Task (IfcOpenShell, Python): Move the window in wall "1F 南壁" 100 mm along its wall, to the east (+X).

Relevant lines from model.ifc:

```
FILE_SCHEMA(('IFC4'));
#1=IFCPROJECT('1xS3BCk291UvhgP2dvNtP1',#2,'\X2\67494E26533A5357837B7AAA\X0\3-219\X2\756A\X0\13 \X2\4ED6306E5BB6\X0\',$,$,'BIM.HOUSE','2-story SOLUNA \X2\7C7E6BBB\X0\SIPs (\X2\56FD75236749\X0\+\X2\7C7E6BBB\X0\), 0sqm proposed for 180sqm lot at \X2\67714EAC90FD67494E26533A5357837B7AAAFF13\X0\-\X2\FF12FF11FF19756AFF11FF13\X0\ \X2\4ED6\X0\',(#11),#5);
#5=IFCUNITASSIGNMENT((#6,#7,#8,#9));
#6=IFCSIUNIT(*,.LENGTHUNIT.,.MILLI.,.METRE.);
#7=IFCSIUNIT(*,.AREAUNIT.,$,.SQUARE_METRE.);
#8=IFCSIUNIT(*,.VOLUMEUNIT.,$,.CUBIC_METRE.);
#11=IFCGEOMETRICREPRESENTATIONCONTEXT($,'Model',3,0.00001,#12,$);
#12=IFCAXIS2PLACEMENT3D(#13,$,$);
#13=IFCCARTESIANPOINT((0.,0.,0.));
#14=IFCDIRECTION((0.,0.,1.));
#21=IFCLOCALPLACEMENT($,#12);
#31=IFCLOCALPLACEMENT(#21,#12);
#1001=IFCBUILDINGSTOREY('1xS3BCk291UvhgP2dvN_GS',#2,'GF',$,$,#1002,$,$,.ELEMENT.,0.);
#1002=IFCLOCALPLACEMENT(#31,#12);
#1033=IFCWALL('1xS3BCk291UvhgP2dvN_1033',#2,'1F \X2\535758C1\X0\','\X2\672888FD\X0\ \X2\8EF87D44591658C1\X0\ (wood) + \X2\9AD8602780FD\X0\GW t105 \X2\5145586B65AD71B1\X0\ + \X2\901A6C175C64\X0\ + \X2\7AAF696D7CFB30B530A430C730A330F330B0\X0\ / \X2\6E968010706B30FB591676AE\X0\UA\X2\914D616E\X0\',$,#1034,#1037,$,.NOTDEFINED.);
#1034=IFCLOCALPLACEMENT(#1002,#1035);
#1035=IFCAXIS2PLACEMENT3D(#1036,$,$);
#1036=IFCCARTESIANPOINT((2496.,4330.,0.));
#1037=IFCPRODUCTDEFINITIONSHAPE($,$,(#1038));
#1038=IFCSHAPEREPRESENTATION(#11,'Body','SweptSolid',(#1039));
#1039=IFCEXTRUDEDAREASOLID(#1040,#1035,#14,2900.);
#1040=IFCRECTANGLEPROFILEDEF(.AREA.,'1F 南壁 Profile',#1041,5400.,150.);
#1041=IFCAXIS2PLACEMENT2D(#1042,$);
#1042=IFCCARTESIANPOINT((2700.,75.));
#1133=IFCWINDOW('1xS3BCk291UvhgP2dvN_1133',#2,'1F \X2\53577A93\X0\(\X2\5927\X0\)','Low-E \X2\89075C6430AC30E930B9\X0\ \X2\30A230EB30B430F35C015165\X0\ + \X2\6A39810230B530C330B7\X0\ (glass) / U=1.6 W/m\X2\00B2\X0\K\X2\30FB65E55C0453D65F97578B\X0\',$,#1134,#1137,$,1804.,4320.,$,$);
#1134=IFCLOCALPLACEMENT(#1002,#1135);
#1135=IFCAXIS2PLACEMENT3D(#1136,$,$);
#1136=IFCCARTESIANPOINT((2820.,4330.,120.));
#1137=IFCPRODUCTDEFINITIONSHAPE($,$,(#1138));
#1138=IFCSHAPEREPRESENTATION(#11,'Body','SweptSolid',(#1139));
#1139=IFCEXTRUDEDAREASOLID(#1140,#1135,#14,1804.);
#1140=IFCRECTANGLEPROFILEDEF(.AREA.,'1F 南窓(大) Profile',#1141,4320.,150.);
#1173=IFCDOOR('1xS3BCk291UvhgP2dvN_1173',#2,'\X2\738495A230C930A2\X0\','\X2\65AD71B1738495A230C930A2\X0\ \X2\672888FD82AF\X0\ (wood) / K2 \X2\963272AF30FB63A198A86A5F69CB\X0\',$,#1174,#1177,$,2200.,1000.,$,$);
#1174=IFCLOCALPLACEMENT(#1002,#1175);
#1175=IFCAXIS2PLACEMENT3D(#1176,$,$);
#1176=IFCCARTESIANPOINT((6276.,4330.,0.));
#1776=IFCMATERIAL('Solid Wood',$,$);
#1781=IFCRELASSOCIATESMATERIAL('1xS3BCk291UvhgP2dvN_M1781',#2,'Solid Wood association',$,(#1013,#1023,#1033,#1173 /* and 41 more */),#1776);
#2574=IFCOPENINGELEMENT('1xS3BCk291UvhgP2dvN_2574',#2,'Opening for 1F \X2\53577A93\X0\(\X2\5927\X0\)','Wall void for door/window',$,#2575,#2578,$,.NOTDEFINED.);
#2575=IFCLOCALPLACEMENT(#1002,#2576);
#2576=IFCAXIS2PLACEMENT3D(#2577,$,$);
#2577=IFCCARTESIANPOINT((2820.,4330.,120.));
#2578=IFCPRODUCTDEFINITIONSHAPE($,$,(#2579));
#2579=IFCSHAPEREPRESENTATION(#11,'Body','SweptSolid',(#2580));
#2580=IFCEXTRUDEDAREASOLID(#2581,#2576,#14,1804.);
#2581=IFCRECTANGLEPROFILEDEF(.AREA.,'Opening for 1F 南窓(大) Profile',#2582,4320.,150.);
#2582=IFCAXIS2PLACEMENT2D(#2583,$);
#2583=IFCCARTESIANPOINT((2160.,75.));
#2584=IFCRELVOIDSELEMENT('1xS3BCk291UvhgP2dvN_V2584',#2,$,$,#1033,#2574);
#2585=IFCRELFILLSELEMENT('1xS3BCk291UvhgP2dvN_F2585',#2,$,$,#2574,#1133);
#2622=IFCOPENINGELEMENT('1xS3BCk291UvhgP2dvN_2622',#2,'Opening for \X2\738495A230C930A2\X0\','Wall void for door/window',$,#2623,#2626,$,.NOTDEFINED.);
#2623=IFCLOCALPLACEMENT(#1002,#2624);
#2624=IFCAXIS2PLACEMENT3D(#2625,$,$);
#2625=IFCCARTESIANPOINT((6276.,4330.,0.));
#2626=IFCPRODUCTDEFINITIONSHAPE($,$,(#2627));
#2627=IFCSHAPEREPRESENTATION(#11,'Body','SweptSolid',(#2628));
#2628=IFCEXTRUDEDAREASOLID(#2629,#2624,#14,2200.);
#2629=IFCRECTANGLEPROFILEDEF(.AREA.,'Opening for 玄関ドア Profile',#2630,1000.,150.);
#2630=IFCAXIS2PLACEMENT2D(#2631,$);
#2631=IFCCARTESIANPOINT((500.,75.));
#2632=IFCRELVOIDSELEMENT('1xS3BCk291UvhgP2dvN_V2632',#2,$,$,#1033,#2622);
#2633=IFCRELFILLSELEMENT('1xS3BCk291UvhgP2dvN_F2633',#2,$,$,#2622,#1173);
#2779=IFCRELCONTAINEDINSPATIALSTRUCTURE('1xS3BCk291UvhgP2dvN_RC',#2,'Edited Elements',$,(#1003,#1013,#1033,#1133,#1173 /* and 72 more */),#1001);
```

```python
import ifcopenshell
import ifcopenshell.api.geometry
import ifcopenshell.util.placement
import ifcopenshell.util.unit

model = ifcopenshell.open("model.ifc")
unit_scale = ifcopenshell.util.unit.calculate_unit_scale(model)

window = model.by_guid("1xS3BCk291UvhgP2dvN_1133")
opening = window.FillsVoids[0].RelatingOpeningElement
wall = opening.VoidsElements[0].RelatingBuildingElement

wall_matrix = ifcopenshell.util.placement.get_local_placement(wall.ObjectPlacement)
shift = wall_matrix[:3, 0] * 0.1 / unit_scale
before = ifcopenshell.util.placement.get_local_placement(window.ObjectPlacement)[:3, 3].copy()

# The window is not placed relative to its opening, so move both.
for product in (opening, window):
    matrix = ifcopenshell.util.placement.get_local_placement(product.ObjectPlacement)
    matrix[:3, 3] += shift
    ifcopenshell.api.geometry.edit_object_placement(model, product=product, matrix=matrix, is_si=False)

after = ifcopenshell.util.placement.get_local_placement(window.ObjectPlacement)[:3, 3]
print("window moved by", (after - before).round(3) + 0.0)

model.write("model_v2.ifc")
```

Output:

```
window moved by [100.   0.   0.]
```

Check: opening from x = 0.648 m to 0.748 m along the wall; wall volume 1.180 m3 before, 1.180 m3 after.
